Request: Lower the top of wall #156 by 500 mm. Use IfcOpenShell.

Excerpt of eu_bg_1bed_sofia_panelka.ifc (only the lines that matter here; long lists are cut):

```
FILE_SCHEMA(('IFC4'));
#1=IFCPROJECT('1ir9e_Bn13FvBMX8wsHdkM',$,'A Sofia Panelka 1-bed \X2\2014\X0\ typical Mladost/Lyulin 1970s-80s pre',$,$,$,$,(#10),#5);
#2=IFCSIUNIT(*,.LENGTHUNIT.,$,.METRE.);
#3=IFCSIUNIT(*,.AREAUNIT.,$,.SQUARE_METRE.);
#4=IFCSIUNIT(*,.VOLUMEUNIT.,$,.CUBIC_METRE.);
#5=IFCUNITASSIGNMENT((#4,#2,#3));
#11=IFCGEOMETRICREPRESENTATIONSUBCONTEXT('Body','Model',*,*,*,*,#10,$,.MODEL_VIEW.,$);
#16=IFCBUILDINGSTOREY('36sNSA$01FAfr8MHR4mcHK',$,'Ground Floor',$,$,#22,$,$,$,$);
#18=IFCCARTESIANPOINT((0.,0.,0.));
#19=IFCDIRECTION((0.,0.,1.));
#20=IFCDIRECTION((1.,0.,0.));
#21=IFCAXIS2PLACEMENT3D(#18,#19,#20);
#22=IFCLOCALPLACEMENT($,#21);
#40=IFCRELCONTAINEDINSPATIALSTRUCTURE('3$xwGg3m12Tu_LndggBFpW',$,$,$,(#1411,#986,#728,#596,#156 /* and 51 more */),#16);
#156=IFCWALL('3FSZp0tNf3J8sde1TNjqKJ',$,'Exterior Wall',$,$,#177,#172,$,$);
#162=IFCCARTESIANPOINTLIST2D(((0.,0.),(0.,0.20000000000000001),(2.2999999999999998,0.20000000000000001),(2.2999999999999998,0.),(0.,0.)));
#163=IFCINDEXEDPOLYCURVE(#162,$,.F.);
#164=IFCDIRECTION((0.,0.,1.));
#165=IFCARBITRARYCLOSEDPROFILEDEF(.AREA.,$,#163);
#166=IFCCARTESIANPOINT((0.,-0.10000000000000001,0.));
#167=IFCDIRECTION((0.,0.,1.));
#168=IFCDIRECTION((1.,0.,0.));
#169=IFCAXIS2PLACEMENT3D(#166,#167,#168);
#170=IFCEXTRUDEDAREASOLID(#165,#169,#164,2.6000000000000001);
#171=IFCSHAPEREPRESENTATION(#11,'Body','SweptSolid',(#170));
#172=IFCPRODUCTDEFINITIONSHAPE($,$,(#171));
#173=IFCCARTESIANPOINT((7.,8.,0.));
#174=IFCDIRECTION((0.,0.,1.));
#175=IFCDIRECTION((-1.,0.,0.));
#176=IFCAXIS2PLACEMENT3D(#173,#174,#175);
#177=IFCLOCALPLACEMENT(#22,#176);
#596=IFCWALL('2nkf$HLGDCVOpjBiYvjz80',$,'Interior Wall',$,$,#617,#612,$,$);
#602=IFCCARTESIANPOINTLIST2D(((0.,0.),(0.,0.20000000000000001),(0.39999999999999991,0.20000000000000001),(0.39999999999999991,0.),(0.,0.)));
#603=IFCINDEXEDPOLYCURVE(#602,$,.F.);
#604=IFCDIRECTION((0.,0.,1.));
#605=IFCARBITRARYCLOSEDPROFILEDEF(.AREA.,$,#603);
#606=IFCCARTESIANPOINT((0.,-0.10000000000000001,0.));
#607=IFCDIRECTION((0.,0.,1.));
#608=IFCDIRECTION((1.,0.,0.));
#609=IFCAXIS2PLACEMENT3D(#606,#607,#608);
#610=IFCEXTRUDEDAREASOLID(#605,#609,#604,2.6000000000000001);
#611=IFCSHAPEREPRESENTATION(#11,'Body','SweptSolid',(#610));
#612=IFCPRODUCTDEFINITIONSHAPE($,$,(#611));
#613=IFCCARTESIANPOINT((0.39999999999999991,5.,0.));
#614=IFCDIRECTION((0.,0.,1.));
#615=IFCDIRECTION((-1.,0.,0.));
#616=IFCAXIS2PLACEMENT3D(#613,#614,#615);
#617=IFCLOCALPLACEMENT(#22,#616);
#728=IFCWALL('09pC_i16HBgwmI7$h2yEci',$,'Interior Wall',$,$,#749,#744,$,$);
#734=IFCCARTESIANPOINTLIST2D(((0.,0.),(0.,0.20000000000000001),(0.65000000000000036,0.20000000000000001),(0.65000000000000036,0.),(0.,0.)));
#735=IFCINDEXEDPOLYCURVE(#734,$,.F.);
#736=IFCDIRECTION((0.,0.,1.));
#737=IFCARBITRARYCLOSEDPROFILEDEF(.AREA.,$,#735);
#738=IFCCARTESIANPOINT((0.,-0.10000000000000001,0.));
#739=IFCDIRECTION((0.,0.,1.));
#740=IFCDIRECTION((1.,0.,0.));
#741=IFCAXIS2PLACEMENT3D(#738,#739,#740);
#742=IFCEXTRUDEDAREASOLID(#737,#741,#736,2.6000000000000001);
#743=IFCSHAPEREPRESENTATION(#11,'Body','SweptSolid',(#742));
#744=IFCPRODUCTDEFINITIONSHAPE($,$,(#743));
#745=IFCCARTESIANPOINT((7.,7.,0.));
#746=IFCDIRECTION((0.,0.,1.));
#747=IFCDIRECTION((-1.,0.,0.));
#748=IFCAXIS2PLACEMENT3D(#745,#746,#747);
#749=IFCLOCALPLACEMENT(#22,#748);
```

```python
import ifcopenshell
import ifcopenshell.geom
import ifcopenshell.util.representation
import ifcopenshell.util.shape
import ifcopenshell.util.unit

model = ifcopenshell.open("eu_bg_1bed_sofia_panelka.ifc")
unit_scale = ifcopenshell.util.unit.calculate_unit_scale(model)
settings = ifcopenshell.geom.settings()


def volume(element):
    """Net volume in cubic metres, openings subtracted."""
    shape = ifcopenshell.geom.create_shape(settings, element)
    return ifcopenshell.util.shape.get_volume(shape.geometry)


wall = model.by_id(156)
before = volume(wall)

body = ifcopenshell.util.representation.get_representation(wall, "Model", "Body")
solid = body.Items[0]
old_height = solid.Depth
solid.Depth -= 0.5 / unit_scale
after = volume(wall)

print(f"height {old_height:g} -> {solid.Depth:g}, volume {before:.3f} -> {after:.3f} m3")

model.write("eu_bg_1bed_sofia_panelka-out.ifc")
```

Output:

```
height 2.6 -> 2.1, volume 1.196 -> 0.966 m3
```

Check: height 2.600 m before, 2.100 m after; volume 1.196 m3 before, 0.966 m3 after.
